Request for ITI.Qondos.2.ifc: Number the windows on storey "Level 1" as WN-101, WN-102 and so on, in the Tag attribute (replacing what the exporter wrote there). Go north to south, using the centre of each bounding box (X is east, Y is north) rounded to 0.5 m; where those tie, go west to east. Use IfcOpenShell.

First a look at what the model holds.

```python
import ifcopenshell
import ifcopenshell.util.element
import ifcopenshell.util.placement

model = ifcopenshell.open("ITI.Qondos.2.ifc")
print(model.schema)
storey = next(s for s in model.by_type("IfcBuildingStorey") if s.Name == "Level 1")
windows = [e for e in ifcopenshell.util.element.get_decomposition(storey) if e.is_a("IfcWindow")]
for e in sorted(windows, key=lambda e: e.id()):
    origin = ifcopenshell.util.placement.get_local_placement(e.ObjectPlacement)[:3, 3]
    print(e.id(), e.Tag, e.Name, origin.round(2) + 0.0, sep=" | ")
```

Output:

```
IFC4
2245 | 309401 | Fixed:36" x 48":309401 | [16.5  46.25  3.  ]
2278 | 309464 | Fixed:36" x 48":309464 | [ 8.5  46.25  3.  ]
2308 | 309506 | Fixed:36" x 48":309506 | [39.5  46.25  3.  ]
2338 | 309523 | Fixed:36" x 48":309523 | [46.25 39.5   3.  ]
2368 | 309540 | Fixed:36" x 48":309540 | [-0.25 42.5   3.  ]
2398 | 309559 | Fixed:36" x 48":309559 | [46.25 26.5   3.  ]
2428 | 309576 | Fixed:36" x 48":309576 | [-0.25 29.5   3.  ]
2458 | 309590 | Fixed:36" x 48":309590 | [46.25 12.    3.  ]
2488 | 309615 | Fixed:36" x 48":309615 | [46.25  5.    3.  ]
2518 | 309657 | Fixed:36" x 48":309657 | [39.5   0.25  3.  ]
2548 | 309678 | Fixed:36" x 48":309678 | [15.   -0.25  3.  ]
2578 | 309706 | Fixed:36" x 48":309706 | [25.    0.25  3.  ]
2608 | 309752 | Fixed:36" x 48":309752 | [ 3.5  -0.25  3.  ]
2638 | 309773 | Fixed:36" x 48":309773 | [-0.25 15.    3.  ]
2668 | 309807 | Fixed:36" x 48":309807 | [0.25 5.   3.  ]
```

```python
import ifcopenshell
import ifcopenshell.geom
import ifcopenshell.util.element
import ifcopenshell.util.shape

model = ifcopenshell.open("ITI.Qondos.2.ifc")
settings = ifcopenshell.geom.settings()
settings.set("use-world-coords", True)


def centre(element):
    shape = ifcopenshell.geom.create_shape(settings, element)
    return ifcopenshell.util.shape.get_bbox_centroid(shape.geometry)


storey = next(s for s in model.by_type("IfcBuildingStorey") if s.Name == "Level 1")
windows = [e for e in ifcopenshell.util.element.get_decomposition(storey) if e.is_a("IfcWindow")]

# Insertion points can sit at a corner or the storey origin, so sort by the geometry (in metres).
centres = {e: centre(e) for e in windows}
windows.sort(key=lambda e: (-round(centres[e][1] / 0.5), centres[e][0]))

for i, e in enumerate(windows, start=1):
    number = f"WN-1{i:02d}"
    e.Tag = number
    print(e.id(), number)

model.write("ITI.Qondos.2_rev.ifc")
```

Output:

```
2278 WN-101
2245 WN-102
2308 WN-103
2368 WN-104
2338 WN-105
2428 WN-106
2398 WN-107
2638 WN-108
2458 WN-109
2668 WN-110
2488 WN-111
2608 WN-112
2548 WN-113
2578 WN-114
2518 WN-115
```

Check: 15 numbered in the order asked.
